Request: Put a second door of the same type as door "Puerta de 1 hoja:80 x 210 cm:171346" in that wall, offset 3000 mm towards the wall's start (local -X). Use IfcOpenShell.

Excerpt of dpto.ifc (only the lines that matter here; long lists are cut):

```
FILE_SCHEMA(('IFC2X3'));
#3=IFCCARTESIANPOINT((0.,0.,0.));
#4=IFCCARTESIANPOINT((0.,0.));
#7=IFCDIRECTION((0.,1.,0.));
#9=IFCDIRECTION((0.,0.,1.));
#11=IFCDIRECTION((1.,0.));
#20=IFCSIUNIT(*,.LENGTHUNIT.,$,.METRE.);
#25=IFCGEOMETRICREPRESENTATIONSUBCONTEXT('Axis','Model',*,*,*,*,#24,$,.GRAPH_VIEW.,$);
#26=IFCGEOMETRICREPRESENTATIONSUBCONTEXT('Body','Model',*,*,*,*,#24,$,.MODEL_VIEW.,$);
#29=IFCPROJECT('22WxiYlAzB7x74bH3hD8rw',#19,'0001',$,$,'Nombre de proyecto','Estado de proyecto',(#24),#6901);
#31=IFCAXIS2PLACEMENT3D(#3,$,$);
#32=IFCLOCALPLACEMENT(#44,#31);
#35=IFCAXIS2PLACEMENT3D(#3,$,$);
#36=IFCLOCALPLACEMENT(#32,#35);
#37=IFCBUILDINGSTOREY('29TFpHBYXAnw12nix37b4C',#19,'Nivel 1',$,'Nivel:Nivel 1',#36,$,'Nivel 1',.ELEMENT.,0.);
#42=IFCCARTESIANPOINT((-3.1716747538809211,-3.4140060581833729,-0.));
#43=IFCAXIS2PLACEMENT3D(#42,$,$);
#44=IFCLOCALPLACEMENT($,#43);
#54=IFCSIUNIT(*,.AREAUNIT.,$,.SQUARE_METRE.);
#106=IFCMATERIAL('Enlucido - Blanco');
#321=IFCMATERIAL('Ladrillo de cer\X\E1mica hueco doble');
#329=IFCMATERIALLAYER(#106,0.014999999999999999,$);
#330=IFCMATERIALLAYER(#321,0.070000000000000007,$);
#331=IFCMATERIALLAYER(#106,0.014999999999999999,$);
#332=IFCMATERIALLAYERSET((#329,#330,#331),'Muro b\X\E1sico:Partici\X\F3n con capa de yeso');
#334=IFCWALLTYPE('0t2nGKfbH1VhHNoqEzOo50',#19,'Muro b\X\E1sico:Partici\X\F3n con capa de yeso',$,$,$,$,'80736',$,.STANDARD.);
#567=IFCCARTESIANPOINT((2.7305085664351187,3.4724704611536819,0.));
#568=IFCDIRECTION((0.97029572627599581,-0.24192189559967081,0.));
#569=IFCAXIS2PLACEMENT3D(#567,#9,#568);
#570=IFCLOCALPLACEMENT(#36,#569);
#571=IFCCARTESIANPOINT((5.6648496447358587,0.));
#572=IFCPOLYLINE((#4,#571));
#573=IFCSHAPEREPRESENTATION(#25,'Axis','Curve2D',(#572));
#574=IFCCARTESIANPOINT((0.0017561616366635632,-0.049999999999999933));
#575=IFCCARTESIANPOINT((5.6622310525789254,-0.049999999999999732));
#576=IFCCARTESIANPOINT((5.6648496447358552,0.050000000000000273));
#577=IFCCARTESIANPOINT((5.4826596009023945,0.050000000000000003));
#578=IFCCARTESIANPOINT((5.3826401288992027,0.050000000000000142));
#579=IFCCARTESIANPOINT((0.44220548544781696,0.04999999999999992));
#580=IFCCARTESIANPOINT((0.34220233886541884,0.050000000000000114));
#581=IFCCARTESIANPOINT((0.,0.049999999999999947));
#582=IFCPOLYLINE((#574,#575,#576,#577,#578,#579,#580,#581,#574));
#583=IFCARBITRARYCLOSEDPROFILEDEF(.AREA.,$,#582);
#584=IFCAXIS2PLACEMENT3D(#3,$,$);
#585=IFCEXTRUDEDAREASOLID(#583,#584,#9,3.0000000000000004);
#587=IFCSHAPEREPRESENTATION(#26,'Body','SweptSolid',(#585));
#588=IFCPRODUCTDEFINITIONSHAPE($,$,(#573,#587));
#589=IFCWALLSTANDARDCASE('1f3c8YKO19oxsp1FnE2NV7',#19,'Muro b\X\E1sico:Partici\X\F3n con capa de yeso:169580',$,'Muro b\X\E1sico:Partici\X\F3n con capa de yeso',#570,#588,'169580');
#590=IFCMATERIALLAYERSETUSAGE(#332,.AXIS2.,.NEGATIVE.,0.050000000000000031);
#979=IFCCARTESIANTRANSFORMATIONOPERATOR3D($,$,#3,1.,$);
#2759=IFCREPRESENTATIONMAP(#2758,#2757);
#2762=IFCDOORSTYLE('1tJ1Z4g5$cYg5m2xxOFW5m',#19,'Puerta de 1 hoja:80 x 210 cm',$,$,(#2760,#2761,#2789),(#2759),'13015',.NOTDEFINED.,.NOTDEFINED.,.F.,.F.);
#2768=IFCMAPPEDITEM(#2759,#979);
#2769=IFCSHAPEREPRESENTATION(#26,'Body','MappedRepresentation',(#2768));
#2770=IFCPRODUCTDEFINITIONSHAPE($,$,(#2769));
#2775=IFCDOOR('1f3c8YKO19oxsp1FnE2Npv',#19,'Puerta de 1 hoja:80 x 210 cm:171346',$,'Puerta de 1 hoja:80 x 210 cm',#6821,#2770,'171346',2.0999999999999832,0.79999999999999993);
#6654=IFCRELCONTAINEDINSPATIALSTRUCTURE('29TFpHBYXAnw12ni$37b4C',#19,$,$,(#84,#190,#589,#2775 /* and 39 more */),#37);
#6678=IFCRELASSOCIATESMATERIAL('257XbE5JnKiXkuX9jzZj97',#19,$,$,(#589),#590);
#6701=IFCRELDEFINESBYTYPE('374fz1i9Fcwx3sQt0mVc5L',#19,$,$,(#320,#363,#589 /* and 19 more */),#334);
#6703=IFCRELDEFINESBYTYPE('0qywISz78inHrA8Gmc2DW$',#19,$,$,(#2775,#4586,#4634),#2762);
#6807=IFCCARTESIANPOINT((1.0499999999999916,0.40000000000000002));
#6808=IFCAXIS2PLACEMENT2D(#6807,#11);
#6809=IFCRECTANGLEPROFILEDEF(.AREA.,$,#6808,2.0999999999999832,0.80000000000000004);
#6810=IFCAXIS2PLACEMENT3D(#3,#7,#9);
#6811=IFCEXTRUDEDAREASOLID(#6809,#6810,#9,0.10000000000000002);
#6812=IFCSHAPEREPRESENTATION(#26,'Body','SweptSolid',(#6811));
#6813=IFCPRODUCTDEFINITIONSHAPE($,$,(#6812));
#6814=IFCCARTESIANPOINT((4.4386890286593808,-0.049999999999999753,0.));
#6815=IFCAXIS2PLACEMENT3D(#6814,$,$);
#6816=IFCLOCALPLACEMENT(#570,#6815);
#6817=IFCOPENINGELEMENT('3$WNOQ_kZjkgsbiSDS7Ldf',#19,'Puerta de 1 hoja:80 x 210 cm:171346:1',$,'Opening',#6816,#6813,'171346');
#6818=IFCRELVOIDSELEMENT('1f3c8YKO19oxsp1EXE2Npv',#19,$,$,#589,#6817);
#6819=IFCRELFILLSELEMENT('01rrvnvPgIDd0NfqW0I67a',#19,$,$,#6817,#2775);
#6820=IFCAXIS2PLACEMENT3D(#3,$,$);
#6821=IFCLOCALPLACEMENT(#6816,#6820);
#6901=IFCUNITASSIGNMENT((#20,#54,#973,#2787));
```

```python
import ifcopenshell
import ifcopenshell.api.feature
import ifcopenshell.api.geometry
import ifcopenshell.api.root
import ifcopenshell.geom
import ifcopenshell.util.element
import ifcopenshell.util.placement
import ifcopenshell.util.shape
import ifcopenshell.util.unit

model = ifcopenshell.open("dpto.ifc")
unit_scale = ifcopenshell.util.unit.calculate_unit_scale(model)
settings = ifcopenshell.geom.settings()


def volume(element):
    """Net volume in cubic metres, openings subtracted."""
    shape = ifcopenshell.geom.create_shape(settings, element)
    return ifcopenshell.util.shape.get_volume(shape.geometry)


def reuse_history(source, copy):
    """copy_class also copies each property set's owner history, people and application; keep the originals."""
    for rel in copy.IsDefinedBy:
        if rel.is_a("IfcRelDefinesByProperties") and (history := rel.RelatingPropertyDefinition.OwnerHistory):
            rel.RelatingPropertyDefinition.OwnerHistory = source.OwnerHistory
            ifcopenshell.util.element.remove_deep2(model, history)


door = model.by_guid("1f3c8YKO19oxsp1FnE2Npv")
opening = door.FillsVoids[0].RelatingOpeningElement
wall = opening.VoidsElements[0].RelatingBuildingElement
before = volume(wall)
shift = ifcopenshell.util.placement.get_local_placement(wall.ObjectPlacement)[:3, 0] * -3 / unit_scale

# copy_class copies the void relationship, type, container and properties, but no geometry.
new_opening = ifcopenshell.api.root.copy_class(model, product=opening)
new_opening.Representation = ifcopenshell.util.element.copy_deep(
    model, opening.Representation, exclude=["IfcGeometricRepresentationContext", "IfcRepresentationMap"]
)
new_opening.Name = "Puerta de 1 hoja:80 x 210 cm"
new_opening.Tag = None
new_door = ifcopenshell.api.root.copy_class(model, product=door)
new_door.Representation = ifcopenshell.util.element.copy_deep(
    model, door.Representation, exclude=["IfcGeometricRepresentationContext", "IfcRepresentationMap"]
)
new_door.Name = "Puerta de 1 hoja:80 x 210 cm"
new_door.Tag = None
reuse_history(door, new_door)
fills = ifcopenshell.api.feature.add_filling(model, opening=new_opening, element=new_door)
fills.OwnerHistory = new_door.OwnerHistory  # required in IFC2X3

for old, new in ((opening, new_opening), (door, new_door)):
    matrix = ifcopenshell.util.placement.get_local_placement(old.ObjectPlacement)
    matrix[:3, 3] += shift
    ifcopenshell.api.geometry.edit_object_placement(model, product=new, matrix=matrix, is_si=False)

after = volume(wall)

print(f"wall volume {before:.3f} -> {after:.3f} m3")

model.write("dpto_v2.ifc")
```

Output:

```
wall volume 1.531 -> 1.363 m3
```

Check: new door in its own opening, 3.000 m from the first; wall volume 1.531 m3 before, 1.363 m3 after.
